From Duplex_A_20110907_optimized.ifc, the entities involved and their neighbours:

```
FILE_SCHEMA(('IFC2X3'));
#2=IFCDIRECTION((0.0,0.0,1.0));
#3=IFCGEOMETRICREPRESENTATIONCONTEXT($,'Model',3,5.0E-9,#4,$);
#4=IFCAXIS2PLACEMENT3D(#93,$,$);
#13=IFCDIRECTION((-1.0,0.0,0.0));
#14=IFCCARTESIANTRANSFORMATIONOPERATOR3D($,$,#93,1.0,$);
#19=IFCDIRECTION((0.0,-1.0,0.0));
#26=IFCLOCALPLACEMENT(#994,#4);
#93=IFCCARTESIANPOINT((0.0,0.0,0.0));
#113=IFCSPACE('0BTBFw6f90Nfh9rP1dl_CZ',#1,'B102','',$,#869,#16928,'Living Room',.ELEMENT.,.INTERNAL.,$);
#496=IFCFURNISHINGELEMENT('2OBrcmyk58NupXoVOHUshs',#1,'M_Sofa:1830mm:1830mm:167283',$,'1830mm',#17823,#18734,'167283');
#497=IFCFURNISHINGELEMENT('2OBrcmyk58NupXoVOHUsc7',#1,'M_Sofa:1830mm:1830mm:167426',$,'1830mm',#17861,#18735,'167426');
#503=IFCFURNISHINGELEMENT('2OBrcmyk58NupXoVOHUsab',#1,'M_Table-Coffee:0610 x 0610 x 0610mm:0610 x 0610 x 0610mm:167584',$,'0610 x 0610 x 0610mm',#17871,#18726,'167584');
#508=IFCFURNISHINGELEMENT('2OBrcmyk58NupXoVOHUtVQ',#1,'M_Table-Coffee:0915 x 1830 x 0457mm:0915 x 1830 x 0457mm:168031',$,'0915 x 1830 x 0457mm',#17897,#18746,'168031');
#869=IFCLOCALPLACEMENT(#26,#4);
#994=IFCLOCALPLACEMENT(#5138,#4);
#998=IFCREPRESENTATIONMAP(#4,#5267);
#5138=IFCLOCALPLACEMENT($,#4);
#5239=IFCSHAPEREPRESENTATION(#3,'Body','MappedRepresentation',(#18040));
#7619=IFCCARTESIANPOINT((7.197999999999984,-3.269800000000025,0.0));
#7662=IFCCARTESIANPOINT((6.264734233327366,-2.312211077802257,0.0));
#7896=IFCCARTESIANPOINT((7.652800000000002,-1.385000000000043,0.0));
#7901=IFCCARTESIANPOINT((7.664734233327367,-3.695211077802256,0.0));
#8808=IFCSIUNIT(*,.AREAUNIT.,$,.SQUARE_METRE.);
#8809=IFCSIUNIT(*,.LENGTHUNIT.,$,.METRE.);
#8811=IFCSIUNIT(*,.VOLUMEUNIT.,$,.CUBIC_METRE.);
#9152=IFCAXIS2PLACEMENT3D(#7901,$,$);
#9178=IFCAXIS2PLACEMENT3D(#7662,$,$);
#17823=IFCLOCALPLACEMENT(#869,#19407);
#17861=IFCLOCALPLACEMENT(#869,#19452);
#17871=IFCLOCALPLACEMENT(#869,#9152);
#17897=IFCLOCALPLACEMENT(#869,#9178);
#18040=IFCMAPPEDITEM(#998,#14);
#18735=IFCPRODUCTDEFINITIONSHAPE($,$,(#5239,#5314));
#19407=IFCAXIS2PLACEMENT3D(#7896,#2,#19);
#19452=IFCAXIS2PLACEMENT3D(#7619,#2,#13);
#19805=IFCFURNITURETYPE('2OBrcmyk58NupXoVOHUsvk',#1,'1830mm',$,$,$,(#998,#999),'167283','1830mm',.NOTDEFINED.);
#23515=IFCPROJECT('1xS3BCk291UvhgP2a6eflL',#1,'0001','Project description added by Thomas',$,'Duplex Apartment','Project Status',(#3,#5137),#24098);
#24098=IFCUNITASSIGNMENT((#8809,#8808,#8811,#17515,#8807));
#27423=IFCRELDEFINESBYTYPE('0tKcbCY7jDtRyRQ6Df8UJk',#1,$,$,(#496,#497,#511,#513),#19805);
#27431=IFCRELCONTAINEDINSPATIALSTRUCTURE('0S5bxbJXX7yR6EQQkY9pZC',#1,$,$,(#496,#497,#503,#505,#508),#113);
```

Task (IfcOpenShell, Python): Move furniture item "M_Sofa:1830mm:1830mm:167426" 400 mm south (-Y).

```python
import ifcopenshell
import ifcopenshell.api.geometry
import ifcopenshell.util.placement

model = ifcopenshell.open("Duplex_A_20110907_optimized.ifc")

item = model.by_guid("2OBrcmyk58NupXoVOHUsc7")
matrix = ifcopenshell.util.placement.get_local_placement(item.ObjectPlacement)
matrix[1, 3] -= 0.4
ifcopenshell.api.geometry.edit_object_placement(model, product=item, matrix=matrix, is_si=False)

print(ifcopenshell.util.placement.get_local_placement(item.ObjectPlacement).round(3) + 0.0)

model.write("Duplex_A_20110907_optimized_edited.ifc")
```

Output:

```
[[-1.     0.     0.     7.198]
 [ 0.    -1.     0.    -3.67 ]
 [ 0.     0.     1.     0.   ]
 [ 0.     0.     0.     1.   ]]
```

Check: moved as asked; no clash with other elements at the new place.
